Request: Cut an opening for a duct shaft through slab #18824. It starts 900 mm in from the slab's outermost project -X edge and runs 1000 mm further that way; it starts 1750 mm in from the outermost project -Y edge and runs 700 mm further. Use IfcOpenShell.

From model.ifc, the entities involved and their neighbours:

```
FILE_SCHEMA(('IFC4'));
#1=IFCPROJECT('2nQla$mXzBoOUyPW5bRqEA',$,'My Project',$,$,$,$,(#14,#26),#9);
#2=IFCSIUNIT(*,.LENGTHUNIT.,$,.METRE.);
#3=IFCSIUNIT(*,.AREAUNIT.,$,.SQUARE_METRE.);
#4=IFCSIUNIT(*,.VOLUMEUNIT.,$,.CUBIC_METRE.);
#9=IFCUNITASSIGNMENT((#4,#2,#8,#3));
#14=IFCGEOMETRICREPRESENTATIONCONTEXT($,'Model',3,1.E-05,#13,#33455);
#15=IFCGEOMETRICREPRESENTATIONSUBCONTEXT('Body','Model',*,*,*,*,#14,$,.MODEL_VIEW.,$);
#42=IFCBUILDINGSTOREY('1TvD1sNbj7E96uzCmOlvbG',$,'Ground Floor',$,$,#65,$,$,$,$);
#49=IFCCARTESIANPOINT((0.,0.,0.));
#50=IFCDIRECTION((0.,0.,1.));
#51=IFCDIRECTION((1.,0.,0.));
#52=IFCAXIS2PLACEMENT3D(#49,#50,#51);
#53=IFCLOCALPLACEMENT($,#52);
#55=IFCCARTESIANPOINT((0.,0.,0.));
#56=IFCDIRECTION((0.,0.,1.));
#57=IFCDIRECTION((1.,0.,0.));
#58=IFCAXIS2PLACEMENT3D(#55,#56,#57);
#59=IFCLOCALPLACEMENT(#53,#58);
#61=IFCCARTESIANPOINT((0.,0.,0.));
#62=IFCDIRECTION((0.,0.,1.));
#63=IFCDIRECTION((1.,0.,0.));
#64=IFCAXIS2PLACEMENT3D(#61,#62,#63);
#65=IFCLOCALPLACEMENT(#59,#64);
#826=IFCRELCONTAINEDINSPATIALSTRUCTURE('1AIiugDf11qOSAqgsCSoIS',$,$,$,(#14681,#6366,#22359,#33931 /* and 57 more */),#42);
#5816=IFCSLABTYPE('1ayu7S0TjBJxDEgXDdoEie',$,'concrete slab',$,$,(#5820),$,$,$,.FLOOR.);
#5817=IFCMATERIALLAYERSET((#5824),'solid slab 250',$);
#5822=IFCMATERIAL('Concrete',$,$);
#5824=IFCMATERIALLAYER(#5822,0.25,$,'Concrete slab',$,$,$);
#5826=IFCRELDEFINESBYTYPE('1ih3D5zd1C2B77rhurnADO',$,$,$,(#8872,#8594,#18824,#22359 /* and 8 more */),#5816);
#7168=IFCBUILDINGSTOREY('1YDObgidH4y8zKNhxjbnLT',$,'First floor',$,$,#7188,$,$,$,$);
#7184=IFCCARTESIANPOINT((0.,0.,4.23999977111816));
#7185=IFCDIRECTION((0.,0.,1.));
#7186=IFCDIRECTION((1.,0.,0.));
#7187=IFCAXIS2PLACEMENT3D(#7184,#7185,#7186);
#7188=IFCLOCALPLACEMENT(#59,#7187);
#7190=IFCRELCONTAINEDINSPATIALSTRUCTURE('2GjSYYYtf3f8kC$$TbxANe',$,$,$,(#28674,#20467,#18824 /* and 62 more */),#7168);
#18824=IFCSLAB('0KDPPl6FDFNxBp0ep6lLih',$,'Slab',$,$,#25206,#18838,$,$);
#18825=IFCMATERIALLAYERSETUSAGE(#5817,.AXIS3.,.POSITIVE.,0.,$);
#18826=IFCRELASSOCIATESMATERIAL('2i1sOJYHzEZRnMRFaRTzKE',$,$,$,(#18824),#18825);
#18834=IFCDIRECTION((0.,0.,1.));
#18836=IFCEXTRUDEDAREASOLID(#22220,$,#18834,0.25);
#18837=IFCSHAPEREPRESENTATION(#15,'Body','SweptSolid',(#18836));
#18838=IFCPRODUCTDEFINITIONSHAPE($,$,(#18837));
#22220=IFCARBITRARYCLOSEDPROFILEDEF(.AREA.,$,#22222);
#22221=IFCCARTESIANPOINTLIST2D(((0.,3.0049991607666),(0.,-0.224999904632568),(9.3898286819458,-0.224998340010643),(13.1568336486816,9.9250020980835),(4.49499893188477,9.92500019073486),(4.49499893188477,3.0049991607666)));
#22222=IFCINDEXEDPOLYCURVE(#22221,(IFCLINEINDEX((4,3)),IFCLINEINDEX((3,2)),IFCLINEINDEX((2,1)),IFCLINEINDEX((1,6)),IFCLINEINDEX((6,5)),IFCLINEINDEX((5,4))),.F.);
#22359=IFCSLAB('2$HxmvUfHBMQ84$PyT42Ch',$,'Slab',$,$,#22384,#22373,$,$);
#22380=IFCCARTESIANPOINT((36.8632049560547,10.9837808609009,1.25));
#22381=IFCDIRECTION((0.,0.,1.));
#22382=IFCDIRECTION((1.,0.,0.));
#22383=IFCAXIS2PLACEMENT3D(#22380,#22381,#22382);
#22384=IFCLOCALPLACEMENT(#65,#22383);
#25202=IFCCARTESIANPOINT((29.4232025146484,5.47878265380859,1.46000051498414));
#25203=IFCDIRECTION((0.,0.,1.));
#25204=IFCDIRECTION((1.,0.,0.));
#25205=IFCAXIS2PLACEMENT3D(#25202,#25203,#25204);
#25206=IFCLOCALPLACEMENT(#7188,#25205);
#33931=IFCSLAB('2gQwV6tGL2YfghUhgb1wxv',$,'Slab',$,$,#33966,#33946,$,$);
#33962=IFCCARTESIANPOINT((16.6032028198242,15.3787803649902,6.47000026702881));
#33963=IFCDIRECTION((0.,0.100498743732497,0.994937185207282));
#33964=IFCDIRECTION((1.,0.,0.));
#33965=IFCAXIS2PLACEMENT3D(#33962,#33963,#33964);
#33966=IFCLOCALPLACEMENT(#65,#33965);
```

```python
import numpy as np
import ifcopenshell
import ifcopenshell.api.feature
import ifcopenshell.api.geometry
import ifcopenshell.api.root
import ifcopenshell.geom
import ifcopenshell.util.placement
import ifcopenshell.util.representation
import ifcopenshell.util.shape
import ifcopenshell.util.unit

model = ifcopenshell.open("model.ifc")
unit_scale = ifcopenshell.util.unit.calculate_unit_scale(model)
settings = ifcopenshell.geom.settings()


def volume(element):
    """Net volume in cubic metres, openings subtracted."""
    shape = ifcopenshell.geom.create_shape(settings, element)
    return ifcopenshell.util.shape.get_volume(shape.geometry)


slab = model.by_guid("0KDPPl6FDFNxBp0ep6lLih")
before = volume(slab)

# Extent in the slab's own axes, in metres. The edges named are its -X and -Y sides.
slab_shape = ifcopenshell.geom.create_shape(settings, slab)
vertices = ifcopenshell.util.shape.get_vertices(slab_shape.geometry)
x_min, y_min, bottom = vertices.min(axis=0)
top = vertices[:, 2].max()

opening = ifcopenshell.api.root.create_entity(model, ifc_class="IfcOpeningElement", name="Duct shaft opening", predefined_type="OPENING")
context = ifcopenshell.util.representation.get_context(model, "Model", "Body", "MODEL_VIEW")
width, depth = 1, 0.7
outline = [(0.0, 0.0), (width, 0.0), (width, depth), (0.0, depth), (0.0, 0.0)]
# Overshoot both faces by 50 mm so the cut is clean.
shape = ifcopenshell.api.geometry.add_slab_representation(
    model, context=context, depth=top - bottom + 0.1, polyline=outline
)
ifcopenshell.api.geometry.assign_representation(model, product=opening, representation=shape)

matrix = ifcopenshell.util.placement.get_local_placement(slab.ObjectPlacement)
matrix[:, 3] = matrix @ np.append(np.array([x_min + 0.9, y_min + 1.75, bottom - 0.05]) / unit_scale, 1.0)
ifcopenshell.api.geometry.edit_object_placement(model, product=opening, matrix=matrix, is_si=False)
ifcopenshell.api.feature.add_feature(model, feature=opening, element=slab)

after = volume(slab)

print(f"slab volume {before:.3f} -> {after:.3f} m3")

model.write("model_v2.ifc")
```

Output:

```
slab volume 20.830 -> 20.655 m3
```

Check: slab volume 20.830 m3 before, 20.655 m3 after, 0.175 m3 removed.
